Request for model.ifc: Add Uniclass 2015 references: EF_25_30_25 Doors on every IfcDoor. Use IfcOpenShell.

First a look at what the model holds.

```python
import ifcopenshell

model = ifcopenshell.open("model.ifc")
print(model.schema)
print("classifications:", [c.Name for c in model.by_type("IfcClassification")])
for ifc_class in ("IfcDoor", "IfcRoof", "IfcStair", "IfcWall", "IfcWindow"):
    print(ifc_class, len(model.by_type(ifc_class)))
```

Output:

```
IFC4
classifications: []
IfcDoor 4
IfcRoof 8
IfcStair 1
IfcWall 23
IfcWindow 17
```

```python
import ifcopenshell
import ifcopenshell.api.classification

model = ifcopenshell.open("model.ifc")

system = ifcopenshell.api.classification.add_classification(model, classification="Uniclass 2015")

codes = {
    "IfcDoor": ("EF_25_30_25", "Doors"),
}
for ifc_class, (code, name) in codes.items():
    products = model.by_type(ifc_class)
    ifcopenshell.api.classification.add_reference(
        model, products=products, classification=system, identification=code, name=name
    )
    print(code, len(products))

model.write("model_rev.ifc")
```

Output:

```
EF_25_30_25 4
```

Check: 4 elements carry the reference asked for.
